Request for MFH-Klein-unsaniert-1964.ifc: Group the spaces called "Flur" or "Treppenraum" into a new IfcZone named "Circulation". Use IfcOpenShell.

First a look at what the model holds.

```python
import ifcopenshell

model = ifcopenshell.open("MFH-Klein-unsaniert-1964.ifc")
print(model.schema)
seen = {}
for space in model.by_type("IfcSpace"):
    seen[space.Name] = seen.get(space.Name, 0) + 1
for name, count in sorted(seen.items(), key=str):
    print(count, "x", name)
print("zones:", [z.Name for z in model.by_type("IfcZone")][:20])
```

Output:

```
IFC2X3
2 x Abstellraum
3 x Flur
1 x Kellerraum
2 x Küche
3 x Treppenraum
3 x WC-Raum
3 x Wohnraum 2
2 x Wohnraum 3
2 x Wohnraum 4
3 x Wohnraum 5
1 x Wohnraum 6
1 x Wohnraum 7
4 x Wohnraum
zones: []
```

```python
import ifcopenshell
import ifcopenshell.api.group
import ifcopenshell.api.root

model = ifcopenshell.open("MFH-Klein-unsaniert-1964.ifc")

names = {"Flur", "Treppenraum"}
spaces = [s for s in model.by_type("IfcSpace") if s.Name in names]

zone = ifcopenshell.api.root.create_entity(model, ifc_class="IfcZone", name="Circulation")
ifcopenshell.api.group.assign_group(model, products=spaces, group=zone)
print(len(spaces), "spaces in", zone.Name)

model.write("MFH-Klein-unsaniert-1964_v2.ifc")
```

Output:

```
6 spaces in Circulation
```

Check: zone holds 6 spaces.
